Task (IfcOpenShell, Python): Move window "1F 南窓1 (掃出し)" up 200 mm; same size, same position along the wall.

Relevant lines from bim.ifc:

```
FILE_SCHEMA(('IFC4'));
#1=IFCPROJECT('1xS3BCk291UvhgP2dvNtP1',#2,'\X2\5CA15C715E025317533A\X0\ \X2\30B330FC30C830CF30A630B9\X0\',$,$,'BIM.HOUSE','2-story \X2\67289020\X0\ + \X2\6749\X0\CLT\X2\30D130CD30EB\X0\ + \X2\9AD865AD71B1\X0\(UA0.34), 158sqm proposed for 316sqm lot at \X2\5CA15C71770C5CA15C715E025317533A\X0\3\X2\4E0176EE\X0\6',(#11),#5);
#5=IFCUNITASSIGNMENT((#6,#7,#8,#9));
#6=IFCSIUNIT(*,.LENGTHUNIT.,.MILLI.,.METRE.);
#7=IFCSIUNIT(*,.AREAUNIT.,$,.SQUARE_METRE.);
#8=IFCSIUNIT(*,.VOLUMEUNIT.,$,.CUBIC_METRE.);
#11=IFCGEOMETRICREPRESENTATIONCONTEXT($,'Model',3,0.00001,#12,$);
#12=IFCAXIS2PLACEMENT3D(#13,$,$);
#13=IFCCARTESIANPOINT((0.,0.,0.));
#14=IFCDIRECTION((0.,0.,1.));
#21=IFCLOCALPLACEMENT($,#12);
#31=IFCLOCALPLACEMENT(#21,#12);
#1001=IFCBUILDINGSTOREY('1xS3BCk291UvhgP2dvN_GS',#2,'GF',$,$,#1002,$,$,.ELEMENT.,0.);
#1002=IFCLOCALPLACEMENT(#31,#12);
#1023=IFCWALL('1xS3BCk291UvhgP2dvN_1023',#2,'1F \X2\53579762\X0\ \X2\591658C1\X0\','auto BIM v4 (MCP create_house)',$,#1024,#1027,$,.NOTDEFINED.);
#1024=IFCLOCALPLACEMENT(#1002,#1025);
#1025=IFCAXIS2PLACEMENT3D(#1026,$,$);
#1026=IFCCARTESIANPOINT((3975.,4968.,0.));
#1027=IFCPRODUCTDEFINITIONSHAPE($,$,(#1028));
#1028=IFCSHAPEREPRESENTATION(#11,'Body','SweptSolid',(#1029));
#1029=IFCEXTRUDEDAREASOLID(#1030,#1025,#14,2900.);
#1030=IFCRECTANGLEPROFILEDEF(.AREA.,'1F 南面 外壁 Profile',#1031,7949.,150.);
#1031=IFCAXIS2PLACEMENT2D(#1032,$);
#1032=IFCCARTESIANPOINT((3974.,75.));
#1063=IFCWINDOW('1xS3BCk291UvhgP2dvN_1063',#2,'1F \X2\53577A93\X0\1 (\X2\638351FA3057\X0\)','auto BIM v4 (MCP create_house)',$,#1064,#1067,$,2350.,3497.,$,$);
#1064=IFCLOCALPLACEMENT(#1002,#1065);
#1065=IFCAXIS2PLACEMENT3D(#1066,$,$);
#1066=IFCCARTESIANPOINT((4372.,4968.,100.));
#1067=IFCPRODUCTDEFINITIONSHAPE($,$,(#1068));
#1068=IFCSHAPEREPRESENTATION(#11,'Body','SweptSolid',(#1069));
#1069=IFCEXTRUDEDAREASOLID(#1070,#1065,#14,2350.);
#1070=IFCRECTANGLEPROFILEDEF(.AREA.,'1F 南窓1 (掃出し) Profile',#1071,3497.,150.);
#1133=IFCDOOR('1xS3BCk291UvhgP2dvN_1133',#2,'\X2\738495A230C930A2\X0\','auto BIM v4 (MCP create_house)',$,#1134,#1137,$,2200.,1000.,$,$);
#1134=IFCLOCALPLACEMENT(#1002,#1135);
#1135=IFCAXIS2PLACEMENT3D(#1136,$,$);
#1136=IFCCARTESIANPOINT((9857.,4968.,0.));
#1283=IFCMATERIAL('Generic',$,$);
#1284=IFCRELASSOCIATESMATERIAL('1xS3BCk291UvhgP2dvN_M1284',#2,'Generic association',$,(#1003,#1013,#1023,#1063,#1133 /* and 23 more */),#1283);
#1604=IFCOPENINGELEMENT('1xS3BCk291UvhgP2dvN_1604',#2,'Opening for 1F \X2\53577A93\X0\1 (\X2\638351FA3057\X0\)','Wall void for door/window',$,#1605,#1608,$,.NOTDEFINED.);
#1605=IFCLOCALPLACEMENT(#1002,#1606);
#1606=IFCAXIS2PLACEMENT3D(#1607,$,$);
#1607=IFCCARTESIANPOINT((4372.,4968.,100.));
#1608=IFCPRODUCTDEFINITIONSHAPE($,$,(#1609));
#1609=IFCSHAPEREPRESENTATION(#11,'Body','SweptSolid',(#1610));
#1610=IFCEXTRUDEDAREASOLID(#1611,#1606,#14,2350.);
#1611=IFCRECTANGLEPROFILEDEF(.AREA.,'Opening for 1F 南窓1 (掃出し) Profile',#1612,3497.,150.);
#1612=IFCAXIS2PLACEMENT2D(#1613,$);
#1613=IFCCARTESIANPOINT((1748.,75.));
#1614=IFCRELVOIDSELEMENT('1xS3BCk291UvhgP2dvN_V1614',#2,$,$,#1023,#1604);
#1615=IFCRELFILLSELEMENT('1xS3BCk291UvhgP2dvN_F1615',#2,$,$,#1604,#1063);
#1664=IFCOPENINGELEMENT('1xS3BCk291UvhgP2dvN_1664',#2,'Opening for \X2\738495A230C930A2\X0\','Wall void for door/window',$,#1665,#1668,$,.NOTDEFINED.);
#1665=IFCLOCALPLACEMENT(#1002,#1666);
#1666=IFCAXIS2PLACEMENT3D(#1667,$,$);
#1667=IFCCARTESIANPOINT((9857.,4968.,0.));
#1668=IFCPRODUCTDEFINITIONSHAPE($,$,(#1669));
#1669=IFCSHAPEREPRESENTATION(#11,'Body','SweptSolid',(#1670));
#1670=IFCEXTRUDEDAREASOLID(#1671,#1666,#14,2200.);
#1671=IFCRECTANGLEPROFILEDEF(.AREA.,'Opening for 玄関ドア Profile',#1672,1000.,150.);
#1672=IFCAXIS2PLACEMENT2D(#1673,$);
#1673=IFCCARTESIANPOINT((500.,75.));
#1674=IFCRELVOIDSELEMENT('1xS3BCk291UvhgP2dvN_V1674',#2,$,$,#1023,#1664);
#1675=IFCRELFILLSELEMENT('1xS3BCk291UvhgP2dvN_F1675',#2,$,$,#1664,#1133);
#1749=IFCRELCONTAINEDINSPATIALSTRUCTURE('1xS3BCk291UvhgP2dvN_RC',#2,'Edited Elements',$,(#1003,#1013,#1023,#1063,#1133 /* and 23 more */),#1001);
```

```python
import numpy as np
import ifcopenshell
import ifcopenshell.api.geometry
import ifcopenshell.util.placement
import ifcopenshell.util.unit

model = ifcopenshell.open("bim.ifc")
unit_scale = ifcopenshell.util.unit.calculate_unit_scale(model)

window = model.by_guid("1xS3BCk291UvhgP2dvN_1063")
opening = window.FillsVoids[0].RelatingOpeningElement
dz = 0.2 / unit_scale

shift = np.array([0.0, 0.0, dz])
# The window is not placed relative to its opening, so move both.
for product in (opening, window):
    matrix = ifcopenshell.util.placement.get_local_placement(product.ObjectPlacement)
    matrix[:3, 3] += shift
    ifcopenshell.api.geometry.edit_object_placement(model, product=product, matrix=matrix, is_si=False)

print(f"moved by {dz * unit_scale:+.3f} m")

model.write("bim_rev.ifc")
```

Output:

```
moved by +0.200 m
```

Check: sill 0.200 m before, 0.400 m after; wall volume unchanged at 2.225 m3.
